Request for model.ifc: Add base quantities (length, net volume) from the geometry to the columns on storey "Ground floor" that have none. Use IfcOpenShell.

First a look at what the model holds.

```python
import ifcopenshell
import ifcopenshell.util.element
import ifcopenshell.util.unit

model = ifcopenshell.open("model.ifc")
print(model.schema)
for unit_type in ("LENGTHUNIT", "AREAUNIT", "VOLUMEUNIT"):
    print(unit_type, ifcopenshell.util.unit.calculate_unit_scale(model, unit_type))
storey = next(s for s in model.by_type("IfcBuildingStorey") if s.Name == "Ground floor")
columns = [e for e in ifcopenshell.util.element.get_decomposition(storey) if e.is_a("IfcColumn")]
for e in sorted(columns, key=lambda e: e.id()):
    print(e.id(), e.is_a(), e.Name, list(ifcopenshell.util.element.get_psets(e, qtos_only=True)), sep=" | ")
```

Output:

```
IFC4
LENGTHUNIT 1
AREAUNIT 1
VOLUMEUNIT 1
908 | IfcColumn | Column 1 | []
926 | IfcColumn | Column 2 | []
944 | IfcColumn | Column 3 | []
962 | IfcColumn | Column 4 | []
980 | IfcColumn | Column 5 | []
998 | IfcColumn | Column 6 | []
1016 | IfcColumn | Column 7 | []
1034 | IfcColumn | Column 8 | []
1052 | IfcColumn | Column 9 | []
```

```python
import ifcopenshell
import ifcopenshell.api.pset
import ifcopenshell.geom
import ifcopenshell.util.element
import ifcopenshell.util.shape
import ifcopenshell.util.unit

model = ifcopenshell.open("model.ifc")
unit_scale = ifcopenshell.util.unit.calculate_unit_scale(model)
volume_scale = ifcopenshell.util.unit.calculate_unit_scale(model, "VOLUMEUNIT")
settings = ifcopenshell.geom.settings()

storey = next(s for s in model.by_type("IfcBuildingStorey") if s.Name == "Ground floor")
columns = [e for e in ifcopenshell.util.element.get_decomposition(storey) if e.is_a("IfcColumn")]

for e in sorted(columns, key=lambda e: e.id()):
    if ifcopenshell.util.element.get_psets(e, qtos_only=True, should_inherit=False):
        continue
    # Geometry comes back in metres, in the element's own axes.
    shape = ifcopenshell.geom.create_shape(settings, e)
    values = {
        "Length": ifcopenshell.util.shape.get_z(shape.geometry) / unit_scale,
        "NetVolume": ifcopenshell.util.shape.get_volume(shape.geometry) / volume_scale,
    }
    qto = ifcopenshell.api.pset.add_qto(model, product=e, name="Qto_ColumnBaseQuantities")
    ifcopenshell.api.pset.edit_qto(model, qto=qto, properties=values)
    print(e.id(), {k: round(v, 3) for k, v in values.items()})

model.write("model-out.ifc")
```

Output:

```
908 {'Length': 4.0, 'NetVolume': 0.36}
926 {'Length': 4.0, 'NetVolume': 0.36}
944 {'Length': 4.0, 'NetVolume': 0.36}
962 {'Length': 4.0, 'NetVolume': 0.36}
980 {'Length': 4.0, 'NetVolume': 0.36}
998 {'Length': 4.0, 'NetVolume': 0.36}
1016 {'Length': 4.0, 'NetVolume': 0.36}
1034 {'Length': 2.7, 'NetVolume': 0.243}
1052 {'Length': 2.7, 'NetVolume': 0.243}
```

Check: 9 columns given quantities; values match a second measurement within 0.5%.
